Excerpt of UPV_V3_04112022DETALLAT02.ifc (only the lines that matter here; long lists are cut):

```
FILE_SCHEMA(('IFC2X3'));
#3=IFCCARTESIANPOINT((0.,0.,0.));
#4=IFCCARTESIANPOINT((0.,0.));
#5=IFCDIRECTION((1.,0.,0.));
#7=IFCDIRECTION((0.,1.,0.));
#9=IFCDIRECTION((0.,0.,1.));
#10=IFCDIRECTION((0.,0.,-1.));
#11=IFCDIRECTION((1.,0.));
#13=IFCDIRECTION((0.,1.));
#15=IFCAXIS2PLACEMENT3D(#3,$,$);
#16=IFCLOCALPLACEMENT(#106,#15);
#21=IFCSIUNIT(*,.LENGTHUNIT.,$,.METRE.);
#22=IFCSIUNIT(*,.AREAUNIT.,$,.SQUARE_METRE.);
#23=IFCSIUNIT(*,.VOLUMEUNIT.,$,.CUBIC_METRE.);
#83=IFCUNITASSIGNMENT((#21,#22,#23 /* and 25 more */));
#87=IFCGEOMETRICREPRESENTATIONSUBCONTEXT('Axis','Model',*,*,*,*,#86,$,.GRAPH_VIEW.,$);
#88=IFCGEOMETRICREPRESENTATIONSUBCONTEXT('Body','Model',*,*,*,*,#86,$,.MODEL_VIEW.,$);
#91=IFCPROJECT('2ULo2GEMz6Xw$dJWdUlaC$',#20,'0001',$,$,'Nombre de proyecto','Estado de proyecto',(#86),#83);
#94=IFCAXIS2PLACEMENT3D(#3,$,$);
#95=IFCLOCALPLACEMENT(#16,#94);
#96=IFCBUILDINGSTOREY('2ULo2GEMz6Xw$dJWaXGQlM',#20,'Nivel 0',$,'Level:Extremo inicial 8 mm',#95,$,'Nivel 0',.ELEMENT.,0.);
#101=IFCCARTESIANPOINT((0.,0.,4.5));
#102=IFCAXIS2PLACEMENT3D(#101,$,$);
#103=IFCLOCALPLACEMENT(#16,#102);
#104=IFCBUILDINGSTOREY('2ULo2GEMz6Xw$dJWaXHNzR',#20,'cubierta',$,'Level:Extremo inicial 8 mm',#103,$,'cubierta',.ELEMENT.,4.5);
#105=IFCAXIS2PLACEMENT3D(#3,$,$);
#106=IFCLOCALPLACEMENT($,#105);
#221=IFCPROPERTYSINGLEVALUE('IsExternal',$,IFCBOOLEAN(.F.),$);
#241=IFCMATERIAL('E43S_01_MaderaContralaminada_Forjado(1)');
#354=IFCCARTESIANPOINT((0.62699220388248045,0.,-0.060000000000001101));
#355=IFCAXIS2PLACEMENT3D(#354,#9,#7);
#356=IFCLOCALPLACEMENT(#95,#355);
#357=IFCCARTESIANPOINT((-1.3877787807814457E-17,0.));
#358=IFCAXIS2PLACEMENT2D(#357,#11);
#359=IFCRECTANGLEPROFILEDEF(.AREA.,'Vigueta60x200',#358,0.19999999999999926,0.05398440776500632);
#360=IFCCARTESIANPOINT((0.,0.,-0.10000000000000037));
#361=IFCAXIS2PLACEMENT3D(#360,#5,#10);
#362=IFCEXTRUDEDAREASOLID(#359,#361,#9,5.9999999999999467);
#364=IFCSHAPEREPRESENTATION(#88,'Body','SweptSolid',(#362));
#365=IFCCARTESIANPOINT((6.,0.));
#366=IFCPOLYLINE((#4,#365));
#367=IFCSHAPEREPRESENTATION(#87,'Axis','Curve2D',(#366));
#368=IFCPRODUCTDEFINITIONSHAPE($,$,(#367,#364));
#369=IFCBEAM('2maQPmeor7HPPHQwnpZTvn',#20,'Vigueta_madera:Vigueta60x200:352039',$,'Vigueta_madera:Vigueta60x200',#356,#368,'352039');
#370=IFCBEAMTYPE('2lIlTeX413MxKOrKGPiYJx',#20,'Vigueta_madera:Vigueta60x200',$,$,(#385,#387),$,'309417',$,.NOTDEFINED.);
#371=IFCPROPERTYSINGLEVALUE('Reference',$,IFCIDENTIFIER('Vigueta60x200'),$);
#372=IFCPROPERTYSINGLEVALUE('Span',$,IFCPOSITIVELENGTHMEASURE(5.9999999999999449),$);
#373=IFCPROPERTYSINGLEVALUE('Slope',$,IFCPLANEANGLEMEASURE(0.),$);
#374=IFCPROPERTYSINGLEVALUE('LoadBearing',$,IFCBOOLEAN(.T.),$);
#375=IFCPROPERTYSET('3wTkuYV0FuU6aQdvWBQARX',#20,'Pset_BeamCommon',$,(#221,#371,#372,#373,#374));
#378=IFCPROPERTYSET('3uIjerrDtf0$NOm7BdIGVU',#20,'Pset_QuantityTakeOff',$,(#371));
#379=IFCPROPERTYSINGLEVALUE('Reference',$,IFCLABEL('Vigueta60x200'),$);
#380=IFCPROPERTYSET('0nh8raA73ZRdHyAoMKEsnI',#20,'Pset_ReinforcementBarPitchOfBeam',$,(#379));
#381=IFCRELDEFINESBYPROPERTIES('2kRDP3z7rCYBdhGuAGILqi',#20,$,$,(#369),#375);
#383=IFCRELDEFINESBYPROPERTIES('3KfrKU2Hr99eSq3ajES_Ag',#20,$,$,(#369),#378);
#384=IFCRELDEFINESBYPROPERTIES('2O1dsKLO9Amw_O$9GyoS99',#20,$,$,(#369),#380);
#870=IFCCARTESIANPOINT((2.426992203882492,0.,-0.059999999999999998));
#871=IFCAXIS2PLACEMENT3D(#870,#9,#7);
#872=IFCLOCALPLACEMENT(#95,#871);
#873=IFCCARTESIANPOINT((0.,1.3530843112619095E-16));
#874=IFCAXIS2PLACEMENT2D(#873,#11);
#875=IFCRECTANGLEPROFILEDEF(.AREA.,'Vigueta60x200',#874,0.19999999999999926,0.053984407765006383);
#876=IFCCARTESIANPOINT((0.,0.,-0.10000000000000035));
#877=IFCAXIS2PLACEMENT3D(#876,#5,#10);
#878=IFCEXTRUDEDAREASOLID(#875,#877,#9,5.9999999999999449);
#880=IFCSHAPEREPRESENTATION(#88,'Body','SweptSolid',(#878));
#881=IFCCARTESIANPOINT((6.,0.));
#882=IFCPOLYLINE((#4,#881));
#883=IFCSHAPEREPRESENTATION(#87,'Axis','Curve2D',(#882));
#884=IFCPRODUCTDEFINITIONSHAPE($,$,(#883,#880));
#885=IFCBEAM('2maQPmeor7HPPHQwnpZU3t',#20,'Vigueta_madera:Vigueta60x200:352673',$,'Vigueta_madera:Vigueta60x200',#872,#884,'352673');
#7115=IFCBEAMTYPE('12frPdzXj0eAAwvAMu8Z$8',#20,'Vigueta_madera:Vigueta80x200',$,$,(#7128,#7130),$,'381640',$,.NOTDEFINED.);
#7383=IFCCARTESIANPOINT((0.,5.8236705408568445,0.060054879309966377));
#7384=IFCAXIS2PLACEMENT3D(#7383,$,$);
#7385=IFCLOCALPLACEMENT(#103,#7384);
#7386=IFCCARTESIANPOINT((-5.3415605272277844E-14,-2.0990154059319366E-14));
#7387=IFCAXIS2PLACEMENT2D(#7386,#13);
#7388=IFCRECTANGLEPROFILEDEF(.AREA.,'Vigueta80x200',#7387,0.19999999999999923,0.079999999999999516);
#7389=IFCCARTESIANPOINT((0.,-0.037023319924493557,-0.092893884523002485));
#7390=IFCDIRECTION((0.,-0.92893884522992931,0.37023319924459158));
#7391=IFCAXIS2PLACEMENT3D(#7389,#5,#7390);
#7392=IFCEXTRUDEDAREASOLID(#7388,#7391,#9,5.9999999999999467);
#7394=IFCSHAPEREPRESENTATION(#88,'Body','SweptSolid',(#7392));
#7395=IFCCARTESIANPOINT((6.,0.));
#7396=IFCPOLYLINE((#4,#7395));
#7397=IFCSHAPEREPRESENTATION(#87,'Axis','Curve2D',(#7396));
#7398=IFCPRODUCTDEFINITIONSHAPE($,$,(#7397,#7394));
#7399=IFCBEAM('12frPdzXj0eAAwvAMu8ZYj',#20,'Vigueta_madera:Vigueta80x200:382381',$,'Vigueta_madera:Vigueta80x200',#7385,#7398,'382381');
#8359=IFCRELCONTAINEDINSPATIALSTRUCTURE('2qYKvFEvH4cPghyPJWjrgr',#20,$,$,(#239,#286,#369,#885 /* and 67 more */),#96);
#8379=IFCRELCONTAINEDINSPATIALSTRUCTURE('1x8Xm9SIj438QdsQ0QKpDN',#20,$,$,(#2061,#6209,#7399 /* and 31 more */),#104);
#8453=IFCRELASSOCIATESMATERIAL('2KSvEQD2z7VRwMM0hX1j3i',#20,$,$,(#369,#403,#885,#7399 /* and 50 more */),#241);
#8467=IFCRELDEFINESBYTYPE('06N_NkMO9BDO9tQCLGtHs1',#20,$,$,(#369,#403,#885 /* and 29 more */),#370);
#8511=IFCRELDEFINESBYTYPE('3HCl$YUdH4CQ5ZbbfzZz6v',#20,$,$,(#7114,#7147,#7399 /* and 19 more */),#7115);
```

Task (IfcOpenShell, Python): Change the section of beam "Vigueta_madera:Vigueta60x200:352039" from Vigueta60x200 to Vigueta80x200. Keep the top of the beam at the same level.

```python
import ifcopenshell
import ifcopenshell.api.pset
import ifcopenshell.api.type
import ifcopenshell.util.element
import ifcopenshell.util.representation

model = ifcopenshell.open("UPV_V3_04112022DETALLAT02.ifc")

member = model.by_id(369)
source = next(p for p in model.by_type("IfcRectangleProfileDef") if p.ProfileName == "Vigueta80x200")

body = ifcopenshell.util.representation.get_representation(member, "Model", "Body")
solid = body.Items[0]
old_profile = solid.SweptArea

# Copy the section's sizes but keep this member's own profile position.
profile = ifcopenshell.util.element.copy(model, source)
# Profiles are centred, so shift by half the change in depth to hold the top.
shift = (old_profile.XDim - profile.XDim) / 2
x, y = old_profile.Position.Location.Coordinates
up = (-1.0, 0.0)  # upwards, in the solid's own plane
location = model.createIfcCartesianPoint((x + up[0] * shift, y + up[1] * shift))
profile.Position = model.createIfcAxis2Placement2D(location, old_profile.Position.RefDirection)
solid.SweptArea = profile
if not model.get_total_inverses(old_profile):
    ifcopenshell.util.element.remove_deep2(model, old_profile)

new_type = model.by_guid("12frPdzXj0eAAwvAMu8Z$8")
ifcopenshell.api.type.assign_type(
    model, related_objects=[member], relating_type=new_type, should_map_representations=False
)
member.Name = member.Name.replace("Vigueta60x200", "Vigueta80x200")
member.ObjectType = "Vigueta_madera:Vigueta80x200"
pset = model.by_id(ifcopenshell.util.element.get_pset(member, "Pset_BeamCommon", should_inherit=False)["id"])
ifcopenshell.api.pset.edit_pset(model, pset=pset, properties={"Reference": "Vigueta80x200"})
pset = model.by_id(ifcopenshell.util.element.get_pset(member, "Pset_QuantityTakeOff", should_inherit=False)["id"])
ifcopenshell.api.pset.edit_pset(model, pset=pset, properties={"Reference": "Vigueta80x200"})
pset = model.by_id(ifcopenshell.util.element.get_pset(member, "Pset_ReinforcementBarPitchOfBeam", should_inherit=False)["id"])
ifcopenshell.api.pset.edit_pset(model, pset=pset, properties={"Reference": "Vigueta80x200"})

print(solid.SweptArea)

model.write("UPV_V3_04112022DETALLAT02_rev.ifc")
```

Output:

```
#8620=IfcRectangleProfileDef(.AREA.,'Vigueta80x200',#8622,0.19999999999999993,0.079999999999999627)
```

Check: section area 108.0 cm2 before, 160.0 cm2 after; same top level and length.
